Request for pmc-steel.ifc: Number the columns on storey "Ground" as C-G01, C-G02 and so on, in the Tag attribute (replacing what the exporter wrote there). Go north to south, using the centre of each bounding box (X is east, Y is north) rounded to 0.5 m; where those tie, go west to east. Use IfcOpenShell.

First a look at what the model holds.

```python
import ifcopenshell
import ifcopenshell.util.element
import ifcopenshell.util.placement

model = ifcopenshell.open("pmc-steel.ifc")
print(model.schema)
storey = next(s for s in model.by_type("IfcBuildingStorey") if s.Name == "Ground")
columns = [e for e in ifcopenshell.util.element.get_decomposition(storey) if e.is_a("IfcColumn")]
for e in sorted(columns, key=lambda e: e.id()):
    origin = ifcopenshell.util.placement.get_local_placement(e.ObjectPlacement)[:3, 3]
    print(e.id(), e.Tag, e.Name, origin.round(2) + 0.0, sep=" | ")
```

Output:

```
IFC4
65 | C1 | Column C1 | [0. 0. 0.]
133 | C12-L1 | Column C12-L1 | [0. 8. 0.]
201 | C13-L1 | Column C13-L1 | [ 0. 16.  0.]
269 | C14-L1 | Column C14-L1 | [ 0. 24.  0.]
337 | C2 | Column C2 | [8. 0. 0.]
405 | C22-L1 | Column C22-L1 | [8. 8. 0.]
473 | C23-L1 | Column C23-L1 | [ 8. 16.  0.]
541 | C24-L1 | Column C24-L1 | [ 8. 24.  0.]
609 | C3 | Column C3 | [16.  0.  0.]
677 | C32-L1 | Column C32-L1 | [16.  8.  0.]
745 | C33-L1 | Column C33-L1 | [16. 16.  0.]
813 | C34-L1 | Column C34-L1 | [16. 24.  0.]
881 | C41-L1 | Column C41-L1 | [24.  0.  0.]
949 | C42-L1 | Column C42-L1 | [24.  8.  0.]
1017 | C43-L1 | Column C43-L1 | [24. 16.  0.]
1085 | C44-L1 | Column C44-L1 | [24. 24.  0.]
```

```python
import ifcopenshell
import ifcopenshell.geom
import ifcopenshell.util.element
import ifcopenshell.util.shape

model = ifcopenshell.open("pmc-steel.ifc")
settings = ifcopenshell.geom.settings()
settings.set("use-world-coords", True)


def centre(element):
    shape = ifcopenshell.geom.create_shape(settings, element)
    return ifcopenshell.util.shape.get_bbox_centroid(shape.geometry)


storey = next(s for s in model.by_type("IfcBuildingStorey") if s.Name == "Ground")
columns = [e for e in ifcopenshell.util.element.get_decomposition(storey) if e.is_a("IfcColumn")]

# Insertion points can sit at a corner or the storey origin, so sort by the geometry (in metres).
centres = {e: centre(e) for e in columns}
columns.sort(key=lambda e: (-round(centres[e][1] / 0.5), centres[e][0]))

for i, e in enumerate(columns, start=1):
    number = f"C-G{i:02d}"
    e.Tag = number
    print(e.id(), number)

model.write("pmc-steel_rev.ifc")
```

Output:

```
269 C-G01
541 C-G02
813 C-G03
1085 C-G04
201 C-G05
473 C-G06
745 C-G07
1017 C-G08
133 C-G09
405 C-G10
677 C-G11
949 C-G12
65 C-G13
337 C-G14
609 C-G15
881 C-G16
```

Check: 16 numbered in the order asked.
